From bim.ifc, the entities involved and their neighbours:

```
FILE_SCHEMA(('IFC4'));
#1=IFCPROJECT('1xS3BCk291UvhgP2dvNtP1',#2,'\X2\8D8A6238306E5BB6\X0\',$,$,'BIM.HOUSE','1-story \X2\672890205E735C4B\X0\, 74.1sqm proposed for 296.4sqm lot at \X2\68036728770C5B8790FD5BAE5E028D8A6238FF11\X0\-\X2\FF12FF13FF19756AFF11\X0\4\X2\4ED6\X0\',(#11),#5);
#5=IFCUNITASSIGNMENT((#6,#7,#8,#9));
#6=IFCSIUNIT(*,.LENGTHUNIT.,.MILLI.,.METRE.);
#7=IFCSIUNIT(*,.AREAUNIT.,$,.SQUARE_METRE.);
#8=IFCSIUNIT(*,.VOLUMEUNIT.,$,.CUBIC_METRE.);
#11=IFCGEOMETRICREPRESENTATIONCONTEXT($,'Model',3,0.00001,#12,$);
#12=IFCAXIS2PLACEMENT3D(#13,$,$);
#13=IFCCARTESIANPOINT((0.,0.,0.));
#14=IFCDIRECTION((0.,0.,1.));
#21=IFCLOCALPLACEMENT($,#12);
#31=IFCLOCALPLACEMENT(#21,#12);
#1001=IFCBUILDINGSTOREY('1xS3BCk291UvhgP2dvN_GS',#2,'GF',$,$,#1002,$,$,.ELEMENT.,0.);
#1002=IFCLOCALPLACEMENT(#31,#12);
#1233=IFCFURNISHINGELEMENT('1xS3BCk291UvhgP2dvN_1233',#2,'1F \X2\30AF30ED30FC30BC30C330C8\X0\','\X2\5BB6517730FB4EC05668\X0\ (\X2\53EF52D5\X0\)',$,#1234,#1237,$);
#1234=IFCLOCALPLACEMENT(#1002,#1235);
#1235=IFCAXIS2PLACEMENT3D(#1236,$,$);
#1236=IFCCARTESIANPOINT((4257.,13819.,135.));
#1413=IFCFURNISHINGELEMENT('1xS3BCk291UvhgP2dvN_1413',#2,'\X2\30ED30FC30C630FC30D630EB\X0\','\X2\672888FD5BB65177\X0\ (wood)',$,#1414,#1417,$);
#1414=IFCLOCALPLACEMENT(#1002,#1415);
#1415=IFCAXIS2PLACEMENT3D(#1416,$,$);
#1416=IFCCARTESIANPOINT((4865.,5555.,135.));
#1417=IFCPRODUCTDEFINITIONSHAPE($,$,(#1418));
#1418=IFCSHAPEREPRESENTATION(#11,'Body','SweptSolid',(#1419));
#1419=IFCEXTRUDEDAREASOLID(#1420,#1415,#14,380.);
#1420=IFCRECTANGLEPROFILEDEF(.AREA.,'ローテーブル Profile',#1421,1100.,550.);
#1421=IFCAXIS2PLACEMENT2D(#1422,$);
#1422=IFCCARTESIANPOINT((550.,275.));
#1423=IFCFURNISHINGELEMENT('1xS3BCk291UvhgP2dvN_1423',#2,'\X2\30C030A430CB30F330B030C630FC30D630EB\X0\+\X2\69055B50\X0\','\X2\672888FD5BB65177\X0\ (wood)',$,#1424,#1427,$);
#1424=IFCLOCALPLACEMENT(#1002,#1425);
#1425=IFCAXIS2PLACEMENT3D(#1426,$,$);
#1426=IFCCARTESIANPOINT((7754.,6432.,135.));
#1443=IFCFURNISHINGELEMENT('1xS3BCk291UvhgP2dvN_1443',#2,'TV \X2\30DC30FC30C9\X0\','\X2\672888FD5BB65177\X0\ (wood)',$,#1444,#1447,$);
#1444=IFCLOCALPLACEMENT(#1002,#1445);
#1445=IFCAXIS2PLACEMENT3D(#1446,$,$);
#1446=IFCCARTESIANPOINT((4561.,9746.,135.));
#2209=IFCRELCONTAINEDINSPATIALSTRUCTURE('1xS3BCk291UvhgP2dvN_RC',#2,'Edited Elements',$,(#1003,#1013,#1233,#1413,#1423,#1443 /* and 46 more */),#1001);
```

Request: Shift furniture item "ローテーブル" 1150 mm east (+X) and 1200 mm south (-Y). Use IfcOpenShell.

```python
import ifcopenshell
import ifcopenshell.api.geometry
import ifcopenshell.util.placement
import ifcopenshell.util.unit

model = ifcopenshell.open("bim.ifc")
unit_scale = ifcopenshell.util.unit.calculate_unit_scale(model)

item = model.by_id(1413)
matrix = ifcopenshell.util.placement.get_local_placement(item.ObjectPlacement)
matrix[0, 3] += 1.15 / unit_scale
matrix[1, 3] -= 1.2 / unit_scale
ifcopenshell.api.geometry.edit_object_placement(model, product=item, matrix=matrix, is_si=False)

print(ifcopenshell.util.placement.get_local_placement(item.ObjectPlacement).round(3) + 0.0)

model.write("bim_edited.ifc")
```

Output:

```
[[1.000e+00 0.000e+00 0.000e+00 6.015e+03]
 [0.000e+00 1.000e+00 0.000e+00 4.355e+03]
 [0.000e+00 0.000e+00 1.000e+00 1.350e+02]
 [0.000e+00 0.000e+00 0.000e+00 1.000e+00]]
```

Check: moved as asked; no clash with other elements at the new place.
